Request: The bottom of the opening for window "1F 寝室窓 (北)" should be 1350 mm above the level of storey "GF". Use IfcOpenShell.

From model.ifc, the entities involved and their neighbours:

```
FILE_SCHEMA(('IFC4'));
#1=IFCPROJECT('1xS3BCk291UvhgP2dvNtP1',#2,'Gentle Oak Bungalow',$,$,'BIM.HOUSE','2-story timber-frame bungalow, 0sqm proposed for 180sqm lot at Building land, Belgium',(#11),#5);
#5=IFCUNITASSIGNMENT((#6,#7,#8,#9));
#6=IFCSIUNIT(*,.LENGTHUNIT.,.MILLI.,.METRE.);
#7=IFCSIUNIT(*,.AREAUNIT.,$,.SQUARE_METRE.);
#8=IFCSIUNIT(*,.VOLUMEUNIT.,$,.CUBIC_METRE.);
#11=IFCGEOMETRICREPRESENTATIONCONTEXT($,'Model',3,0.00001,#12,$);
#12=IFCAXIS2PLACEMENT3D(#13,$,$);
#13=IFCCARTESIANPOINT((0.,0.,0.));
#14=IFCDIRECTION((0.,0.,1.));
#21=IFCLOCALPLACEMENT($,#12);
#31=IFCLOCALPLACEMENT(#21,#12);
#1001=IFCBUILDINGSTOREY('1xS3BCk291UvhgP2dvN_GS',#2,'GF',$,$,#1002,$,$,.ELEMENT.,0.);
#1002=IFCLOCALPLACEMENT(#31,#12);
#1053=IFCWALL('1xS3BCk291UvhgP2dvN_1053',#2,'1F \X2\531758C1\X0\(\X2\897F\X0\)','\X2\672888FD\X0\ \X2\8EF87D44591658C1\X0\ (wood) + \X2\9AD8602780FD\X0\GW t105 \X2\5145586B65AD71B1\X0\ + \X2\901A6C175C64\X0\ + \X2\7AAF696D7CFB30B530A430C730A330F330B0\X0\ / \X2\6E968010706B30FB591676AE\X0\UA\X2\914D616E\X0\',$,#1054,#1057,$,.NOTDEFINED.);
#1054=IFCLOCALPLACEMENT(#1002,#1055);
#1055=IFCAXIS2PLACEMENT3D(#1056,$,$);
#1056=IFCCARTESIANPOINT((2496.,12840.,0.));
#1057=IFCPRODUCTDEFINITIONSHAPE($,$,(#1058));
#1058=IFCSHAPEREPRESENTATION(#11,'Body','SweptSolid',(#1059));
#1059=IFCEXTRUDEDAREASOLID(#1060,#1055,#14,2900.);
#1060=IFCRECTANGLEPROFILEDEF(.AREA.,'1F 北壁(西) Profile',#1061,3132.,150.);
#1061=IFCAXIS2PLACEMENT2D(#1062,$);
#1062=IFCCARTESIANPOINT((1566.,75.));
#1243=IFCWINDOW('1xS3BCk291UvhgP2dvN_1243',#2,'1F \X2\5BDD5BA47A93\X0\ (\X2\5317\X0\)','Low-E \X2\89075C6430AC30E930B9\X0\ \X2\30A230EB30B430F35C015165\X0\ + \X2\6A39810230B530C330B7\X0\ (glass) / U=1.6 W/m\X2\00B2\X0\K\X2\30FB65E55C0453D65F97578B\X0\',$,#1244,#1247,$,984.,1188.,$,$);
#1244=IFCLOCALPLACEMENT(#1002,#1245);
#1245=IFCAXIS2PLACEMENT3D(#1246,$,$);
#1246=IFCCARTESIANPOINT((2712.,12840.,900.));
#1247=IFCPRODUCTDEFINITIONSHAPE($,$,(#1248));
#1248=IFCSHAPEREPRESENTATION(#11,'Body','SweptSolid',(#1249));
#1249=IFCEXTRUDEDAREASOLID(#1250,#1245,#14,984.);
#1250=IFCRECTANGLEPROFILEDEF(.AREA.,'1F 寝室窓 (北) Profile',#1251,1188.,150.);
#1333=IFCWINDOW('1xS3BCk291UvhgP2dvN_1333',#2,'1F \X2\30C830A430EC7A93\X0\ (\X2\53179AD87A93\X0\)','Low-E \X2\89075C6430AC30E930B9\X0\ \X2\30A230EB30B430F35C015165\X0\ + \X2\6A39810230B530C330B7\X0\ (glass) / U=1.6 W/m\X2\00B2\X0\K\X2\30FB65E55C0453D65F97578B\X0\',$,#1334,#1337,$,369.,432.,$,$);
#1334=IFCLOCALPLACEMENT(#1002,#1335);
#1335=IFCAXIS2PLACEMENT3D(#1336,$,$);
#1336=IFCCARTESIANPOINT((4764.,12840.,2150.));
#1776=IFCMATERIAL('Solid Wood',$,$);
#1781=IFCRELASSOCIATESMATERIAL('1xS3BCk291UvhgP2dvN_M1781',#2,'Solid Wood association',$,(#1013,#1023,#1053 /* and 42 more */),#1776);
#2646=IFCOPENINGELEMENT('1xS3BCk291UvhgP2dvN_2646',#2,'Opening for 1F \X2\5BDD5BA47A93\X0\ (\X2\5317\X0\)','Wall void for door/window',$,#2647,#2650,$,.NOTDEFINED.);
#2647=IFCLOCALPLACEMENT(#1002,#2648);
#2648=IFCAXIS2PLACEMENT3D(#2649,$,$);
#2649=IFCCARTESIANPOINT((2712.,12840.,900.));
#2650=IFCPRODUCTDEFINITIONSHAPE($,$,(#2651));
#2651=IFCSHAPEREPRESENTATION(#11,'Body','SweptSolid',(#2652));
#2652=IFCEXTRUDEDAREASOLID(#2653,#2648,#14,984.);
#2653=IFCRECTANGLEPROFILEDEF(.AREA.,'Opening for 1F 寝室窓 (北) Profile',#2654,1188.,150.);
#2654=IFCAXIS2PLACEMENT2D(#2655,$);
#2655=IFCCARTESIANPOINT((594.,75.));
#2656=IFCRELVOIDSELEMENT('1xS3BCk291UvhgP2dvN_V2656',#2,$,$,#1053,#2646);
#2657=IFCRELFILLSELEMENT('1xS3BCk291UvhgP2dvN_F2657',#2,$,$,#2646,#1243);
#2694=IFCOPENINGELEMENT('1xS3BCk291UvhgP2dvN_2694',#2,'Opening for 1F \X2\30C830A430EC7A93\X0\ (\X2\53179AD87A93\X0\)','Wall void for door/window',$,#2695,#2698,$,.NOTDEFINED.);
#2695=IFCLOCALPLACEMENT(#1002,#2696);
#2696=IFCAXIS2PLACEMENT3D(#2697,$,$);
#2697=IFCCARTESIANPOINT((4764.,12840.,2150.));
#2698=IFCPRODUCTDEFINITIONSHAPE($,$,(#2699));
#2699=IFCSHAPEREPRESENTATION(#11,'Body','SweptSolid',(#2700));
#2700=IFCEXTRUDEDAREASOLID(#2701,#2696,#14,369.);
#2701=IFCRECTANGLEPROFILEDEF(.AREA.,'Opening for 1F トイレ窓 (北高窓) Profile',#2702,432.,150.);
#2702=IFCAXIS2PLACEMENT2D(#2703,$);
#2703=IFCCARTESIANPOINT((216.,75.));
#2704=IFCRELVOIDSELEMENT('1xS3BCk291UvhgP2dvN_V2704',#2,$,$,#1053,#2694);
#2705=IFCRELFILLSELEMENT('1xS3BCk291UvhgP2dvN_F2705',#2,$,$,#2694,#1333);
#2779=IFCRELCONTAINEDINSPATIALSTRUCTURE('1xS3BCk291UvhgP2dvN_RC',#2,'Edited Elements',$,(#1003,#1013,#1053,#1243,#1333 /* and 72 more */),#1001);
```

```python
import numpy as np
import ifcopenshell
import ifcopenshell.api.geometry
import ifcopenshell.geom
import ifcopenshell.util.element
import ifcopenshell.util.placement
import ifcopenshell.util.shape
import ifcopenshell.util.unit

model = ifcopenshell.open("model.ifc")
unit_scale = ifcopenshell.util.unit.calculate_unit_scale(model)

window = model.by_guid("1xS3BCk291UvhgP2dvN_1243")
opening = window.FillsVoids[0].RelatingOpeningElement
storey = ifcopenshell.util.element.get_container(window, ifc_class="IfcBuildingStorey")
level = ifcopenshell.util.placement.get_local_placement(storey.ObjectPlacement)[2, 3]

# The opening's origin need not be at the sill, so measure its lowest point.
shape = ifcopenshell.geom.create_shape(ifcopenshell.geom.settings(), opening)
bottom = ifcopenshell.util.shape.get_shape_bottom_elevation(shape, shape.geometry) / unit_scale
dz = level + 1350.0 - bottom

shift = np.array([0.0, 0.0, dz])
# The window is not placed relative to its opening, so move both.
for product in (opening, window):
    matrix = ifcopenshell.util.placement.get_local_placement(product.ObjectPlacement)
    matrix[:3, 3] += shift
    ifcopenshell.api.geometry.edit_object_placement(model, product=product, matrix=matrix, is_si=False)

print(f"moved by {dz * unit_scale:+.3f} m")

model.write("model_updated.ifc")
```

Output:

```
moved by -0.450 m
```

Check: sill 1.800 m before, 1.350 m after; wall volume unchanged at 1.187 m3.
